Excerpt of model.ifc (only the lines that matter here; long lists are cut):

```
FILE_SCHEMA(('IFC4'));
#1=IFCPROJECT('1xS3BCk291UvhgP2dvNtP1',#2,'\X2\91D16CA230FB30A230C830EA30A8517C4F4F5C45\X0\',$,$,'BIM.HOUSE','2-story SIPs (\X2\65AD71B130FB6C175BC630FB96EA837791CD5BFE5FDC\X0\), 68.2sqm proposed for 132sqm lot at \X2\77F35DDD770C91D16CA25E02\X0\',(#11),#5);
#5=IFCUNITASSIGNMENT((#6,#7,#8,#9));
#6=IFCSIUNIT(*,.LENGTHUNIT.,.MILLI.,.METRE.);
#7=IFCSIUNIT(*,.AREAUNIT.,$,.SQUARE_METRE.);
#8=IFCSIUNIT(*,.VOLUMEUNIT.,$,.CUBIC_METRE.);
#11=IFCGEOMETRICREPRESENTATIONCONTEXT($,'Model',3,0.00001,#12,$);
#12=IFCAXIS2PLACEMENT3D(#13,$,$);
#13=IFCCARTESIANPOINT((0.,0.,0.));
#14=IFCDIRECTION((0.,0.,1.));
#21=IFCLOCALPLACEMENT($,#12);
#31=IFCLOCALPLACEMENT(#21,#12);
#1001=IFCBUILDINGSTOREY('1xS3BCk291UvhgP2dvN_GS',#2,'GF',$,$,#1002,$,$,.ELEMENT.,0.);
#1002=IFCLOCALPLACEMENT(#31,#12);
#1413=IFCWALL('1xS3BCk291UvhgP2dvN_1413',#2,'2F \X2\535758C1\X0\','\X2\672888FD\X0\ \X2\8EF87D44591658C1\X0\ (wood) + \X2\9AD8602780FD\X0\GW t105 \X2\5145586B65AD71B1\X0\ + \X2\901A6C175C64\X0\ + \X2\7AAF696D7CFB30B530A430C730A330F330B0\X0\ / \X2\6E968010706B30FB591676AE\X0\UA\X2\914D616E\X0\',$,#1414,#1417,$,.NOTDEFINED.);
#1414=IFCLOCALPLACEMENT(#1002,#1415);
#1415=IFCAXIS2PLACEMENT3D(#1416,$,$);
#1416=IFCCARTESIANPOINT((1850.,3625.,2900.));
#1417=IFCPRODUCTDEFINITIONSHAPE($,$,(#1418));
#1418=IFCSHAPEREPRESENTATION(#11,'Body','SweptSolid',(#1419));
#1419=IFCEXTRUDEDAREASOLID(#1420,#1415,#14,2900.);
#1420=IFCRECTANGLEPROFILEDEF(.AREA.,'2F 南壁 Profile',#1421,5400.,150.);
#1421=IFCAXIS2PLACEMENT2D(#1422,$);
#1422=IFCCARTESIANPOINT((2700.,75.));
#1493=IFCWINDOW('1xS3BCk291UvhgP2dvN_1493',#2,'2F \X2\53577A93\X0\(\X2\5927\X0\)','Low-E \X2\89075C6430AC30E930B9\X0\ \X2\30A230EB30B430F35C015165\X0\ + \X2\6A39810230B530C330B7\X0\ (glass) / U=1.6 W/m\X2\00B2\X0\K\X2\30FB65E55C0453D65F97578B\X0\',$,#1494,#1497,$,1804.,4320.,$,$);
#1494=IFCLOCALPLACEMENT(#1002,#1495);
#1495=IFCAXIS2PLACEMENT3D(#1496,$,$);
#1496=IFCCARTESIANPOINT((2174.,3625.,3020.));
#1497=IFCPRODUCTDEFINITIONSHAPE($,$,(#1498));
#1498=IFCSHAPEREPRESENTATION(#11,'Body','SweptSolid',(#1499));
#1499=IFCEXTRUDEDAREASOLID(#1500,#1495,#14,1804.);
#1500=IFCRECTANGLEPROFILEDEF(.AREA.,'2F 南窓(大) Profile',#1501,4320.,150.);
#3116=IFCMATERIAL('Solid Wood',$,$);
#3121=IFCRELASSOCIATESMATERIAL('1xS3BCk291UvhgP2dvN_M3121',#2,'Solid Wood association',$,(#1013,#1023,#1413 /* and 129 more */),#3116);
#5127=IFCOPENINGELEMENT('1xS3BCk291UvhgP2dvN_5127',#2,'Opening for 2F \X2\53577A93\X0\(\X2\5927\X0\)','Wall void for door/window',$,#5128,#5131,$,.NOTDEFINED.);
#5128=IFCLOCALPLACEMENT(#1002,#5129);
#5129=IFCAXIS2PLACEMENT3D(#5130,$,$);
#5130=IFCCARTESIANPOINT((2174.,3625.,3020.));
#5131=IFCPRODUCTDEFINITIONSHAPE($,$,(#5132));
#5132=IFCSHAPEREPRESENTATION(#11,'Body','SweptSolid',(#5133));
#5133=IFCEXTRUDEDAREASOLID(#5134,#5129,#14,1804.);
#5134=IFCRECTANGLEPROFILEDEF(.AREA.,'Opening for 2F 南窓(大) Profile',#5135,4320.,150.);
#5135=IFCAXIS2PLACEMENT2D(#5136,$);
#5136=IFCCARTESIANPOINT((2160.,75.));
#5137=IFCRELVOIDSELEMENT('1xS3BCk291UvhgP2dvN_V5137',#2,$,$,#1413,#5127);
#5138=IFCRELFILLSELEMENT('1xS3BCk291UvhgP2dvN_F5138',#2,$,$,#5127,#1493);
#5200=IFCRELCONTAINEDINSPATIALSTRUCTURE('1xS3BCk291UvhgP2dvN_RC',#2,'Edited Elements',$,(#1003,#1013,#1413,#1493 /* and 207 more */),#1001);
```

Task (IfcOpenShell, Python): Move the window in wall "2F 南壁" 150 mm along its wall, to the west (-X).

```python
import ifcopenshell
import ifcopenshell.api.geometry
import ifcopenshell.util.placement
import ifcopenshell.util.unit

model = ifcopenshell.open("model.ifc")
unit_scale = ifcopenshell.util.unit.calculate_unit_scale(model)

window = model.by_id(1493)
opening = window.FillsVoids[0].RelatingOpeningElement
wall = opening.VoidsElements[0].RelatingBuildingElement

wall_matrix = ifcopenshell.util.placement.get_local_placement(wall.ObjectPlacement)
shift = wall_matrix[:3, 0] * -0.15 / unit_scale
before = ifcopenshell.util.placement.get_local_placement(window.ObjectPlacement)[:3, 3].copy()

# The window is not placed relative to its opening, so move both.
for product in (opening, window):
    matrix = ifcopenshell.util.placement.get_local_placement(product.ObjectPlacement)
    matrix[:3, 3] += shift
    ifcopenshell.api.geometry.edit_object_placement(model, product=product, matrix=matrix, is_si=False)

after = ifcopenshell.util.placement.get_local_placement(window.ObjectPlacement)[:3, 3]
print("window moved by", (after - before).round(3) + 0.0)

model.write("model-out.ifc")
```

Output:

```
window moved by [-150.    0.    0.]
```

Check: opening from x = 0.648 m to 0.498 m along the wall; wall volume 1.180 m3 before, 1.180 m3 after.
